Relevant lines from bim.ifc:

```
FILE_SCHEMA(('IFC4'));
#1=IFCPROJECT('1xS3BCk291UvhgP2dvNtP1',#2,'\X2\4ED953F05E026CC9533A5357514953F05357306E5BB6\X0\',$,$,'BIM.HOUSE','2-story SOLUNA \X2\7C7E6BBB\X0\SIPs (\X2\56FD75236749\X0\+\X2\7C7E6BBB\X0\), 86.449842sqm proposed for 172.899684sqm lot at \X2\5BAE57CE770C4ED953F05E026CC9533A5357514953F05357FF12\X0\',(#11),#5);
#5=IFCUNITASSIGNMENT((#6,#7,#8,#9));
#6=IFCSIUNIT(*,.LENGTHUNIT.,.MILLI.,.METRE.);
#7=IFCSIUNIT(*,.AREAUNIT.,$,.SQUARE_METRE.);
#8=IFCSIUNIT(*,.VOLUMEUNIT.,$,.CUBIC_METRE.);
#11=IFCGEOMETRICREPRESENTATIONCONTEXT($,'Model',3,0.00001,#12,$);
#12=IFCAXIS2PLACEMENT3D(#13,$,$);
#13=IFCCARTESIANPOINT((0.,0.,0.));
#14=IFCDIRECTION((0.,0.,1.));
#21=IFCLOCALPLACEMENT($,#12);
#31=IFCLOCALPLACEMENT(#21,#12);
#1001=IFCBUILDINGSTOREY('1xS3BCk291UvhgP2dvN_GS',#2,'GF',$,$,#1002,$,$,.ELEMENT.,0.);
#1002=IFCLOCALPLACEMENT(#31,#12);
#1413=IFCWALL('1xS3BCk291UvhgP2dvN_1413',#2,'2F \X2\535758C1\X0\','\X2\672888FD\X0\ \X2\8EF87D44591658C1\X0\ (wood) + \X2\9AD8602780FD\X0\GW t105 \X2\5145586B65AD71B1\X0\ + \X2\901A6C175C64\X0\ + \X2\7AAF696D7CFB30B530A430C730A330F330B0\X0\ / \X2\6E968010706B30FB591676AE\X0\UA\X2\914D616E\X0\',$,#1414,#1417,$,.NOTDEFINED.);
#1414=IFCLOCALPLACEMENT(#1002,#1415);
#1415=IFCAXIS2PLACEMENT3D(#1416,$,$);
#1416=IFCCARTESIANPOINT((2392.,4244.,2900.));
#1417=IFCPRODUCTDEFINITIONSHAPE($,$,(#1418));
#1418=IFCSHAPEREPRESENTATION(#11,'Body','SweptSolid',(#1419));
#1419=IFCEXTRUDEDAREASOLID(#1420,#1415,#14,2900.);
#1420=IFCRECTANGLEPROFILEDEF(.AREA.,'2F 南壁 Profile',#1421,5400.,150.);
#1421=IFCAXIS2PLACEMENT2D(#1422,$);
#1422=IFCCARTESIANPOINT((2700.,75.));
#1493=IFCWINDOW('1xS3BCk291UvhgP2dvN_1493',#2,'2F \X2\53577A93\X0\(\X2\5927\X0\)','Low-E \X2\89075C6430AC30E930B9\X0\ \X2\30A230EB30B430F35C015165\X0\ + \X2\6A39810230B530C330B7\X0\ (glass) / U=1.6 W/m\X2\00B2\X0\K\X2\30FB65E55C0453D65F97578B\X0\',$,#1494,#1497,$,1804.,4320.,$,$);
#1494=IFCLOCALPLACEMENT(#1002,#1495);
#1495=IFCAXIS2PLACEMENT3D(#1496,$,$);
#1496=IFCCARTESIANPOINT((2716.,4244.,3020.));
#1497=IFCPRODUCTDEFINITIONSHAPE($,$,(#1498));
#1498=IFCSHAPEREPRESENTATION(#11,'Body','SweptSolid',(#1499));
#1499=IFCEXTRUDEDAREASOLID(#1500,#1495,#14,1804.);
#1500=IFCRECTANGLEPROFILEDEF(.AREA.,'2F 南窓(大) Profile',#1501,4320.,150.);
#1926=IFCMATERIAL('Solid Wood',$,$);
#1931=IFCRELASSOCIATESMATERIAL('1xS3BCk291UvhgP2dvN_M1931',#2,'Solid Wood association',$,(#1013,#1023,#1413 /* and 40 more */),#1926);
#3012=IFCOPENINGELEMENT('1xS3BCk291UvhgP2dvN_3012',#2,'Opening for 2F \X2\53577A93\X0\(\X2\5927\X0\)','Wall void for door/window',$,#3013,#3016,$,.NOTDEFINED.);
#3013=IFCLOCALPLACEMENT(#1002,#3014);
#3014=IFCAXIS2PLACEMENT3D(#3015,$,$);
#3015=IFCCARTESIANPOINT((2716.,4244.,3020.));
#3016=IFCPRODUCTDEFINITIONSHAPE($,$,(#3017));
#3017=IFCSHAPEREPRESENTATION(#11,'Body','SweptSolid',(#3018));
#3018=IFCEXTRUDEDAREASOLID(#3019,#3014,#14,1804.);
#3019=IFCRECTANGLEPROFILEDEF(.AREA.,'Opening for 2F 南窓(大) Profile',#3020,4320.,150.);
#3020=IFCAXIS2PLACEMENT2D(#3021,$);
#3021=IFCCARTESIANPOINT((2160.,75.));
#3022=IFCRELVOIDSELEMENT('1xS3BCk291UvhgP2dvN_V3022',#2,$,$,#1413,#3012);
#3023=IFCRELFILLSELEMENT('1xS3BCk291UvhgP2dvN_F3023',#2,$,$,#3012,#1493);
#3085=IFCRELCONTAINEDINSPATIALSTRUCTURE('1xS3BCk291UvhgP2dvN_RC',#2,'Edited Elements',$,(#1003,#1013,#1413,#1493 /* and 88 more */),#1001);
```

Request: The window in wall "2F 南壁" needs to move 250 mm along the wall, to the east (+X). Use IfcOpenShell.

```python
import ifcopenshell
import ifcopenshell.api.geometry
import ifcopenshell.util.placement
import ifcopenshell.util.unit

model = ifcopenshell.open("bim.ifc")
unit_scale = ifcopenshell.util.unit.calculate_unit_scale(model)

window = model.by_guid("1xS3BCk291UvhgP2dvN_1493")
opening = window.FillsVoids[0].RelatingOpeningElement
wall = opening.VoidsElements[0].RelatingBuildingElement

wall_matrix = ifcopenshell.util.placement.get_local_placement(wall.ObjectPlacement)
shift = wall_matrix[:3, 0] * 0.25 / unit_scale
before = ifcopenshell.util.placement.get_local_placement(window.ObjectPlacement)[:3, 3].copy()

# The window is not placed relative to its opening, so move both.
for product in (opening, window):
    matrix = ifcopenshell.util.placement.get_local_placement(product.ObjectPlacement)
    matrix[:3, 3] += shift
    ifcopenshell.api.geometry.edit_object_placement(model, product=product, matrix=matrix, is_si=False)

after = ifcopenshell.util.placement.get_local_placement(window.ObjectPlacement)[:3, 3]
print("window moved by", (after - before).round(3) + 0.0)

model.write("bim_rev.ifc")
```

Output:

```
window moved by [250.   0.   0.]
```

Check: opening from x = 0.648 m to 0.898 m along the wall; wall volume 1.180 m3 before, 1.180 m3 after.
